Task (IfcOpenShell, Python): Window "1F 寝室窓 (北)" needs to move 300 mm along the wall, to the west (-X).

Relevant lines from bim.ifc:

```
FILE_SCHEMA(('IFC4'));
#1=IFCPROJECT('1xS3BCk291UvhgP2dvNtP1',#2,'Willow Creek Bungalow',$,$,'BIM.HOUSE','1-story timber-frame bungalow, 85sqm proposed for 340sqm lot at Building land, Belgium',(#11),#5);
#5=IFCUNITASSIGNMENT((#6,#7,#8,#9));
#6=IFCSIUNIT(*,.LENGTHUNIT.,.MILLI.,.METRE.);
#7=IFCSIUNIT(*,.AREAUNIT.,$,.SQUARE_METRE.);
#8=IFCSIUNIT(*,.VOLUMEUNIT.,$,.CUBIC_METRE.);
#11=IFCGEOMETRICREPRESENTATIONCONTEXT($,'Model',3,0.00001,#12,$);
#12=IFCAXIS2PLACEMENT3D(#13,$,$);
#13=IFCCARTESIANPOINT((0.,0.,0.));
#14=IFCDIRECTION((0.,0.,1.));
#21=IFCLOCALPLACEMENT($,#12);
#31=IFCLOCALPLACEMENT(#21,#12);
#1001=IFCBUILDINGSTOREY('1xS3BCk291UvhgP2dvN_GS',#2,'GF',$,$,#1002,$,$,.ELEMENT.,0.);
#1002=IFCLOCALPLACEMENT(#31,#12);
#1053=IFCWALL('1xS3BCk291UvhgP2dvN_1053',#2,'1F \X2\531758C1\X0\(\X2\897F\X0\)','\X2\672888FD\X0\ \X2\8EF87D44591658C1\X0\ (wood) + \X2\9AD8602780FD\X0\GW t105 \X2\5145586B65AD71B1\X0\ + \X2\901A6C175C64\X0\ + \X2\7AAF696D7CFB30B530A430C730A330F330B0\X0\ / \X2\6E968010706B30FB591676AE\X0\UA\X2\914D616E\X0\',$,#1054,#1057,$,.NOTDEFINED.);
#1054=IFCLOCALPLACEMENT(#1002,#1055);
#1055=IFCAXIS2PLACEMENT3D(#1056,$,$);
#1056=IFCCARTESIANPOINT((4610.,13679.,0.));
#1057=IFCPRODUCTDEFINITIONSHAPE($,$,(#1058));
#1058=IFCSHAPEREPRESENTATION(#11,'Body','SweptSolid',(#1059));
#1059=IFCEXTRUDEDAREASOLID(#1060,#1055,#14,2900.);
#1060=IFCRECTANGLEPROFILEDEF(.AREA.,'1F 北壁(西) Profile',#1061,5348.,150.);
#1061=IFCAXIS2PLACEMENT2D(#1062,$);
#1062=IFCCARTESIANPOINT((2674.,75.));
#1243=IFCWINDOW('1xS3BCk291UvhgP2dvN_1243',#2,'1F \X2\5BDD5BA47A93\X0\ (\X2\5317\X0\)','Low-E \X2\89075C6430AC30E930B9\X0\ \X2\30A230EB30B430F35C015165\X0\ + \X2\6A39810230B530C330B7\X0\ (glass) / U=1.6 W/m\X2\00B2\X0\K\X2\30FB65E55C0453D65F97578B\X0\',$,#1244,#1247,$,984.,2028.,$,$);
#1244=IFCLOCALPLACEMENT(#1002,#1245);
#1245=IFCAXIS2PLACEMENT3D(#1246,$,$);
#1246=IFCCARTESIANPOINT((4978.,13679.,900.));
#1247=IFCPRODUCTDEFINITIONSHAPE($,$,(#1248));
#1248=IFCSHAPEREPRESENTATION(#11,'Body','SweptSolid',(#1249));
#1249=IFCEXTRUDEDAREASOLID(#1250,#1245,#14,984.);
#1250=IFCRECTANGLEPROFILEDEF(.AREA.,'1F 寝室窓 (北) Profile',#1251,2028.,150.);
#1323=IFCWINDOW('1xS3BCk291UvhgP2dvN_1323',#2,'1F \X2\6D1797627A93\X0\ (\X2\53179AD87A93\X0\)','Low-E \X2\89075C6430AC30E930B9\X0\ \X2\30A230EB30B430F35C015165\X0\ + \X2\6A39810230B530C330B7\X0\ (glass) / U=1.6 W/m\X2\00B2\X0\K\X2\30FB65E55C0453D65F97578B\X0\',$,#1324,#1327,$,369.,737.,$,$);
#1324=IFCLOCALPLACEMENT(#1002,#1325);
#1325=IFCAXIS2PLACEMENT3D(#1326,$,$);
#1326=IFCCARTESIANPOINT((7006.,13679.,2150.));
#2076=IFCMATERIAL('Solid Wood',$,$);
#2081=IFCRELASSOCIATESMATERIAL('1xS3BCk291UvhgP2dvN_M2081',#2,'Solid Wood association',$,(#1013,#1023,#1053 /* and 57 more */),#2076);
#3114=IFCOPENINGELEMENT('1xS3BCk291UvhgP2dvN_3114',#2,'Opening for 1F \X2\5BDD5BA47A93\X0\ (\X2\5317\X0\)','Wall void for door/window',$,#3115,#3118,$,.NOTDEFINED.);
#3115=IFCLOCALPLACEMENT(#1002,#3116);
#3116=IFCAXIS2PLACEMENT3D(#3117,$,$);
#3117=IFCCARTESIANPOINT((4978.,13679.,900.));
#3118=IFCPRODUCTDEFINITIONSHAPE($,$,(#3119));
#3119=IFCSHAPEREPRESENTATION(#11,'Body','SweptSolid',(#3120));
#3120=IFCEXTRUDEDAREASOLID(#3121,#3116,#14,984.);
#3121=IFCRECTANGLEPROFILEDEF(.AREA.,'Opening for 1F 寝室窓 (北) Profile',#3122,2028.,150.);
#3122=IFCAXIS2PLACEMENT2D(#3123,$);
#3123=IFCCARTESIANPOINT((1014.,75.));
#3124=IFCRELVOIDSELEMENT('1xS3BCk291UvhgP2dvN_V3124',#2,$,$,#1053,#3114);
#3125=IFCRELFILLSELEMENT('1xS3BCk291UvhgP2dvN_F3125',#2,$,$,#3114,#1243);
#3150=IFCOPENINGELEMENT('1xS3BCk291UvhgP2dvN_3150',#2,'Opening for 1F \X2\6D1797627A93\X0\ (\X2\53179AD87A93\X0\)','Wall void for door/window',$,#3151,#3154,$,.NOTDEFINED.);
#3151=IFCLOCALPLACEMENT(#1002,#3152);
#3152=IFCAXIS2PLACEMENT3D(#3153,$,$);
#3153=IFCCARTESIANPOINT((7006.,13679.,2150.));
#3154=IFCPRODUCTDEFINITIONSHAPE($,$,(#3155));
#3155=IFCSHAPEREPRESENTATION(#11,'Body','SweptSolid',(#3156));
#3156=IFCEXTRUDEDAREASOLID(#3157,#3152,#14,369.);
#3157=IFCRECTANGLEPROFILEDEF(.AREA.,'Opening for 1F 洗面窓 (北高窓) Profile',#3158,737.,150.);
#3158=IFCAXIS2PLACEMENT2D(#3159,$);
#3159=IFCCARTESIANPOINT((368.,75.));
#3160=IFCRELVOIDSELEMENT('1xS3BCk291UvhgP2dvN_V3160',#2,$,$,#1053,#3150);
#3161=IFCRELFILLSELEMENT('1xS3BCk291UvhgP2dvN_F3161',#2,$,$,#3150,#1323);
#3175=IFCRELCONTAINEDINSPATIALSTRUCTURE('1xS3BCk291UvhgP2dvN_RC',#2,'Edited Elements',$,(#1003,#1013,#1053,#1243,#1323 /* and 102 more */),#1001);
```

```python
import ifcopenshell
import ifcopenshell.api.geometry
import ifcopenshell.util.placement

model = ifcopenshell.open("bim.ifc")

window = model.by_guid("1xS3BCk291UvhgP2dvN_1243")
opening = window.FillsVoids[0].RelatingOpeningElement
wall = opening.VoidsElements[0].RelatingBuildingElement

wall_matrix = ifcopenshell.util.placement.get_local_placement(wall.ObjectPlacement)
shift = wall_matrix[:3, 0] * -300.0
before = ifcopenshell.util.placement.get_local_placement(window.ObjectPlacement)[:3, 3].copy()

# The window is not placed relative to its opening, so move both.
for product in (opening, window):
    matrix = ifcopenshell.util.placement.get_local_placement(product.ObjectPlacement)
    matrix[:3, 3] += shift
    ifcopenshell.api.geometry.edit_object_placement(model, product=product, matrix=matrix, is_si=False)

after = ifcopenshell.util.placement.get_local_placement(window.ObjectPlacement)[:3, 3]
print("window moved by", (after - before).round(3) + 0.0)

model.write("bim_updated.ifc")
```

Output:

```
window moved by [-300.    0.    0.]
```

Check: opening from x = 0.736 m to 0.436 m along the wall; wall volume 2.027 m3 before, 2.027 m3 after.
